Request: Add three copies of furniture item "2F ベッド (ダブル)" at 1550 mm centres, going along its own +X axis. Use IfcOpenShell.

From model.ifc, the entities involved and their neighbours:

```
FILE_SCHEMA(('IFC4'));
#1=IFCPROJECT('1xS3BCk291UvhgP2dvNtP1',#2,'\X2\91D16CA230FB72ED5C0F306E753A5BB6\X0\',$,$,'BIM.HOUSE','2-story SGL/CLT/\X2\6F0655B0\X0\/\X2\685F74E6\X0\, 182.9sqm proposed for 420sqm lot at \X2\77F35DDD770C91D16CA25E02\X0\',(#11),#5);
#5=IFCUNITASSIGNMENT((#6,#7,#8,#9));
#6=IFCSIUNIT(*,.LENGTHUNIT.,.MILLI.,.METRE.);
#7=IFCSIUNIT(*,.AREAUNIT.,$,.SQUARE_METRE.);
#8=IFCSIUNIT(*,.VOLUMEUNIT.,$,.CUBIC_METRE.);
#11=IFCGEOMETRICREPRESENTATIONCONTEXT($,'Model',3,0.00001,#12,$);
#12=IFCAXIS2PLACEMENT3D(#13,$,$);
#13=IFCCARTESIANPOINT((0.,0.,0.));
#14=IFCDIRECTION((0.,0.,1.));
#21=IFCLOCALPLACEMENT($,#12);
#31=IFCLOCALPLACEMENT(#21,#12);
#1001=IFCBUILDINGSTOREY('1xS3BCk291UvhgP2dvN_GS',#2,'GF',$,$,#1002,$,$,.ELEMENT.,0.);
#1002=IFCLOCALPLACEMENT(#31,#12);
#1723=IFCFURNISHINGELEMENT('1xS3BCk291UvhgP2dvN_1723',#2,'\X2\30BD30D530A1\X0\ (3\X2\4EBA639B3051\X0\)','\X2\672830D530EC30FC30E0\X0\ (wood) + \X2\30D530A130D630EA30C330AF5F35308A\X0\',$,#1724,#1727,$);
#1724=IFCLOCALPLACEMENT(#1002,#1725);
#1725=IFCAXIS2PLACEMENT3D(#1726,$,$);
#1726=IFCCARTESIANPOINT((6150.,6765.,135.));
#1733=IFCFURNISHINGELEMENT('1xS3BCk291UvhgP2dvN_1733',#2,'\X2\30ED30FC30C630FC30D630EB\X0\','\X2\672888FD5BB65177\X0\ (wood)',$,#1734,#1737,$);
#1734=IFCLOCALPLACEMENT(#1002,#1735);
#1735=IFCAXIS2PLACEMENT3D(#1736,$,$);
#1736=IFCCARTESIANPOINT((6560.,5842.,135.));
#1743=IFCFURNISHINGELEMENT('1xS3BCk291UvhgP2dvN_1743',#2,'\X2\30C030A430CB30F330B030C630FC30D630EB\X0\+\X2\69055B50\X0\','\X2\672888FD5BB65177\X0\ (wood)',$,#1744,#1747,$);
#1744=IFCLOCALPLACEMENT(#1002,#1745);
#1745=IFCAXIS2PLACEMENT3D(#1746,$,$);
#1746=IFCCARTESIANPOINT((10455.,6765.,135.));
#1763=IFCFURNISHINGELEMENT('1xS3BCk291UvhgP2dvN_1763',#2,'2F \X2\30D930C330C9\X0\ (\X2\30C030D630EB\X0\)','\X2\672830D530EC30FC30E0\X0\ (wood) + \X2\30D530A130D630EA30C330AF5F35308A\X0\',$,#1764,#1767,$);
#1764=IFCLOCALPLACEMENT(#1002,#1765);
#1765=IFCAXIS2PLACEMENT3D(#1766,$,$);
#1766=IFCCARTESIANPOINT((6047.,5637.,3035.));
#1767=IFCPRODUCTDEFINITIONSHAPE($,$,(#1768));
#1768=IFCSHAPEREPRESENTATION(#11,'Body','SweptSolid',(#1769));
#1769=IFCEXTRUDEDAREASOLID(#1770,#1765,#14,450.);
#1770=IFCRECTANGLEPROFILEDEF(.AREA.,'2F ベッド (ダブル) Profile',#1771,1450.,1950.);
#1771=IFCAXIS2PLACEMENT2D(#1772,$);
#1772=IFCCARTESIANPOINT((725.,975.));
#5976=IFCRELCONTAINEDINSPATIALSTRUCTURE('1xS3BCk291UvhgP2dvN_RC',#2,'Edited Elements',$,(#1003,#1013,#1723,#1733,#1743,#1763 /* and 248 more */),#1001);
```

```python
import ifcopenshell
import ifcopenshell.api.geometry
import ifcopenshell.api.root
import ifcopenshell.util.element
import ifcopenshell.util.placement
import ifcopenshell.util.unit

model = ifcopenshell.open("model.ifc")
unit_scale = ifcopenshell.util.unit.calculate_unit_scale(model)


def reuse_history(source, copy):
    """copy_class also copies each property set's owner history, people and application; keep the originals."""
    for rel in copy.IsDefinedBy:
        if rel.is_a("IfcRelDefinesByProperties") and (history := rel.RelatingPropertyDefinition.OwnerHistory):
            rel.RelatingPropertyDefinition.OwnerHistory = source.OwnerHistory
            ifcopenshell.util.element.remove_deep2(model, history)


source = model.by_guid("1xS3BCk291UvhgP2dvN_1763")
base = ifcopenshell.util.placement.get_local_placement(source.ObjectPlacement)
step = base[:3, 0] * 1.55 / unit_scale

for i in range(1, 4):
    copy = ifcopenshell.api.root.copy_class(model, product=source)
    copy.Representation = ifcopenshell.util.element.copy_deep(
        model, source.Representation, exclude=["IfcGeometricRepresentationContext", "IfcRepresentationMap"]
    )
    reuse_history(source, copy)
    matrix = base.copy()
    matrix[:3, 3] += i * step
    print("added at", matrix[:3, 3].round(3) + 0.0)
    ifcopenshell.api.geometry.edit_object_placement(model, product=copy, matrix=matrix, is_si=False)

model.write("model_edited.ifc")
```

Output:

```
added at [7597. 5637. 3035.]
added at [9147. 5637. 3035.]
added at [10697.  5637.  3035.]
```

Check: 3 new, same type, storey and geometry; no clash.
